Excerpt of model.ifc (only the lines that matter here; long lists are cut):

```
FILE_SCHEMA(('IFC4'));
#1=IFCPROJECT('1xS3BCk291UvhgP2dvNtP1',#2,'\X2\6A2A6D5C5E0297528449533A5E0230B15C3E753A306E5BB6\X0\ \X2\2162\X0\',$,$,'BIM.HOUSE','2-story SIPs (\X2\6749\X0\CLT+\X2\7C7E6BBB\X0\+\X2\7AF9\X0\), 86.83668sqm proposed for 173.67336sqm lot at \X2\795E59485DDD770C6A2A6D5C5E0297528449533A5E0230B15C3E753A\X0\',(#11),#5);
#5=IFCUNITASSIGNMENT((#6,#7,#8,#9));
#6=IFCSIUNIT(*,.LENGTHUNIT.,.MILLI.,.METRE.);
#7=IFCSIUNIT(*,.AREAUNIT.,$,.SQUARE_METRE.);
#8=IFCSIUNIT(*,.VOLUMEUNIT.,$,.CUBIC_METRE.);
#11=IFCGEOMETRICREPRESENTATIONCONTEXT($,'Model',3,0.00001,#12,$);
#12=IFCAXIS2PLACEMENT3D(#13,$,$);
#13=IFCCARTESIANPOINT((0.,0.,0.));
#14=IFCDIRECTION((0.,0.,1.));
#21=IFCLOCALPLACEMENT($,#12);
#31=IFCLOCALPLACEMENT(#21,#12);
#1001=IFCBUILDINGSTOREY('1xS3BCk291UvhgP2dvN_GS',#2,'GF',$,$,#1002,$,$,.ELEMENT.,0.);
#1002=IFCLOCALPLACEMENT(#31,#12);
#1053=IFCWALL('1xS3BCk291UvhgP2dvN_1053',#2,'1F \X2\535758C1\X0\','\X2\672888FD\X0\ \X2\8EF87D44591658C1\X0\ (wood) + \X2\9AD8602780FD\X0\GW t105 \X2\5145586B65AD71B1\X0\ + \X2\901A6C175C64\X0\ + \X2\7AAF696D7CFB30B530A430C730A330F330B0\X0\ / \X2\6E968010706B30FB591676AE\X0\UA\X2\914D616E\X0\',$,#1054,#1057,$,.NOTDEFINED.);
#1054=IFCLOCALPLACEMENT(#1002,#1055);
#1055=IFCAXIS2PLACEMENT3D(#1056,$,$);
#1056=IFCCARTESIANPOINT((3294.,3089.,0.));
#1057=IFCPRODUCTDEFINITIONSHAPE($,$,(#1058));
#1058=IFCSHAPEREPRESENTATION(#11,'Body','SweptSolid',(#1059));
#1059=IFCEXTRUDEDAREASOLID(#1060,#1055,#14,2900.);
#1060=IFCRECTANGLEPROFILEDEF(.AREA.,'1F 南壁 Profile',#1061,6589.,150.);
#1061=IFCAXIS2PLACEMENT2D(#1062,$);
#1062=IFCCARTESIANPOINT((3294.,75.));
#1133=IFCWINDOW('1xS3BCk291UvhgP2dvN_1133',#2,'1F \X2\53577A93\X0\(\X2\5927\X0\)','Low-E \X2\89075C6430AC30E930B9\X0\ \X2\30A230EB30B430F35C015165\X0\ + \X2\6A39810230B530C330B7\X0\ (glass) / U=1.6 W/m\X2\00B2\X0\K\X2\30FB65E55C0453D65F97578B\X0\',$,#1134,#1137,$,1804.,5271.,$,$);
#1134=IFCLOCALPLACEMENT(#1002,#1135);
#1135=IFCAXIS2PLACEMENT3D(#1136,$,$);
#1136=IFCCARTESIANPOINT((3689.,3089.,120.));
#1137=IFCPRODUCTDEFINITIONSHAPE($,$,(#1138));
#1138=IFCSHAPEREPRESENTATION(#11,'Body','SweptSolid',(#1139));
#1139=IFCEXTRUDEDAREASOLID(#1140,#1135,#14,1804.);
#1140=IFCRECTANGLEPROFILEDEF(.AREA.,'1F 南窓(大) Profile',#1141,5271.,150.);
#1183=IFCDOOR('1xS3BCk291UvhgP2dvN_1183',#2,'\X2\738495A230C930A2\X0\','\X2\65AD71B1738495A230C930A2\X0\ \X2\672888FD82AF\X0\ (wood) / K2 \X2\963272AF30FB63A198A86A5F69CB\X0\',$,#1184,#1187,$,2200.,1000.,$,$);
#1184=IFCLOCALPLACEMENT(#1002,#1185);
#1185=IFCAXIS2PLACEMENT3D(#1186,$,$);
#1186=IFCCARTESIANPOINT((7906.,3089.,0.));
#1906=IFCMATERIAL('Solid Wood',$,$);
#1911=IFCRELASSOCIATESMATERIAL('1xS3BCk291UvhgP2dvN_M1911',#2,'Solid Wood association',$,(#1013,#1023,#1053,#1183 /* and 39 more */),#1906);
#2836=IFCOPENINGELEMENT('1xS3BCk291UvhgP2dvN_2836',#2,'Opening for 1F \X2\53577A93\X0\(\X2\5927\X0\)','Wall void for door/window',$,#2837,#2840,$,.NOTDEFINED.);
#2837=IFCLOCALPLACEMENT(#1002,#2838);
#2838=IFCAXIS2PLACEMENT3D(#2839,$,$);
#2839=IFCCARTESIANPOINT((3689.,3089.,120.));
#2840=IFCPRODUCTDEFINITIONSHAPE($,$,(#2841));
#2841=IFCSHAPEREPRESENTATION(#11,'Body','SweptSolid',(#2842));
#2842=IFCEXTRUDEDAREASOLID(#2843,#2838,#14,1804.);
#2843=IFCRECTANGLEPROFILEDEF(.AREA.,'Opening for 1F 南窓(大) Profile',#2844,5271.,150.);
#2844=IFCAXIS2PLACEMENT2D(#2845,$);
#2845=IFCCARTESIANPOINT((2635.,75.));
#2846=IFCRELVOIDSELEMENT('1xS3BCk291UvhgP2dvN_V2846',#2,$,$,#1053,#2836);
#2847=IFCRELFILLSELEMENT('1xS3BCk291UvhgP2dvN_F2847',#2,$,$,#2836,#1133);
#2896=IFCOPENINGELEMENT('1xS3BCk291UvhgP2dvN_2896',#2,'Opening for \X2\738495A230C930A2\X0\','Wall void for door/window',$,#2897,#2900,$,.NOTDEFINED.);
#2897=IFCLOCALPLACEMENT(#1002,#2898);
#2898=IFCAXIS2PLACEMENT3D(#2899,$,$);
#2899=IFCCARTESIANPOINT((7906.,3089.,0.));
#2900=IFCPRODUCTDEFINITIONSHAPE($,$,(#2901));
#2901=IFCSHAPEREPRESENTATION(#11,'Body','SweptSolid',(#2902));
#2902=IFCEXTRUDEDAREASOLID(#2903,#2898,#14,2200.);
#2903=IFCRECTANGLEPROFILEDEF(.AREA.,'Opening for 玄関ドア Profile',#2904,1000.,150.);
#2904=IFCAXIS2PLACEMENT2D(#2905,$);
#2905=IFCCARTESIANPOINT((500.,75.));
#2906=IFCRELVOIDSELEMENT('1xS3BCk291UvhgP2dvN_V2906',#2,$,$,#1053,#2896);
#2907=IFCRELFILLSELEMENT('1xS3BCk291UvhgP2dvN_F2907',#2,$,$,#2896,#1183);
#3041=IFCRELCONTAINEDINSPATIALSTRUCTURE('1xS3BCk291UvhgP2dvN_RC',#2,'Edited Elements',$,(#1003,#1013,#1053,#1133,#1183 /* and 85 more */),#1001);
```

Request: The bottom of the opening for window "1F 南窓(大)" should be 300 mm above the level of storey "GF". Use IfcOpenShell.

```python
import numpy as np
import ifcopenshell
import ifcopenshell.api.geometry
import ifcopenshell.geom
import ifcopenshell.util.element
import ifcopenshell.util.placement
import ifcopenshell.util.shape
import ifcopenshell.util.unit

model = ifcopenshell.open("model.ifc")
unit_scale = ifcopenshell.util.unit.calculate_unit_scale(model)

window = model.by_guid("1xS3BCk291UvhgP2dvN_1133")
opening = window.FillsVoids[0].RelatingOpeningElement
storey = ifcopenshell.util.element.get_container(window, ifc_class="IfcBuildingStorey")
level = ifcopenshell.util.placement.get_local_placement(storey.ObjectPlacement)[2, 3]

# The opening's origin need not be at the sill, so measure its lowest point.
shape = ifcopenshell.geom.create_shape(ifcopenshell.geom.settings(), opening)
bottom = ifcopenshell.util.shape.get_shape_bottom_elevation(shape, shape.geometry) / unit_scale
dz = level + 0.3 / unit_scale - bottom

shift = np.array([0.0, 0.0, dz])
# The window is not placed relative to its opening, so move both.
for product in (opening, window):
    matrix = ifcopenshell.util.placement.get_local_placement(product.ObjectPlacement)
    matrix[:3, 3] += shift
    ifcopenshell.api.geometry.edit_object_placement(model, product=product, matrix=matrix, is_si=False)

print(f"moved by {dz * unit_scale:+.3f} m")

model.write("model_edited.ifc")
```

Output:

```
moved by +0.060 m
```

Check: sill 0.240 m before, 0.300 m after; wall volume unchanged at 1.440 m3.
